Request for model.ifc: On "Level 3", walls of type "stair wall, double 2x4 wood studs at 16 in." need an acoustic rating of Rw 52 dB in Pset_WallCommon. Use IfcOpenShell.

First a look at what the model holds.

```python
import ifcopenshell
import ifcopenshell.util.element

model = ifcopenshell.open("model.ifc")
print(model.schema)
storey = next(s for s in model.by_type("IfcBuildingStorey") if s.Name == "Level 3")
walls = [e for e in ifcopenshell.util.element.get_decomposition(storey) if e.is_a("IfcWall")]
seen = {}
for e in walls:
    element_type = ifcopenshell.util.element.get_type(e)
    key = (element_type.Name if element_type != e and element_type else None, ifcopenshell.util.element.get_pset(e, "Pset_WallCommon", "AcousticRating"))
    seen[key] = seen.get(key, 0) + 1
for (name, value), count in sorted(seen.items(), key=str):
    print(count, "x", name, "|", value)
```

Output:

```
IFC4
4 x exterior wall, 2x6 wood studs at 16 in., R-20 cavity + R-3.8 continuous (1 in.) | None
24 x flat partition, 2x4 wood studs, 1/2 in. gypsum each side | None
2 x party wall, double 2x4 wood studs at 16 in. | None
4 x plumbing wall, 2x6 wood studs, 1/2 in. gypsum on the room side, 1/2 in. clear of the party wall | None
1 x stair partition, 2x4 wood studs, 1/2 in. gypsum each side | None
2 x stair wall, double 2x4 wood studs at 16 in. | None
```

```python
import ifcopenshell
import ifcopenshell.api.pset
import ifcopenshell.util.element

model = ifcopenshell.open("model.ifc")

storey = next(s for s in model.by_type("IfcBuildingStorey") if s.Name == "Level 3")
walls = [e for e in ifcopenshell.util.element.get_decomposition(storey) if e.is_a("IfcWall")]

count = 0
for e in walls:
    element_type = ifcopenshell.util.element.get_type(e)
    if element_type in (None, e) or element_type.Name != "stair wall, double 2x4 wood studs at 16 in.":
        continue
    # add_pset returns the element's existing set when there is one.
    pset = ifcopenshell.api.pset.add_pset(model, product=e, name="Pset_WallCommon")
    ifcopenshell.api.pset.edit_pset(model, pset=pset, properties={"AcousticRating": "Rw 52 dB"})
    count += 1

print(count, "walls updated")

model.write("model_rev.ifc")
```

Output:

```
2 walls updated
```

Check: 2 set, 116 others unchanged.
